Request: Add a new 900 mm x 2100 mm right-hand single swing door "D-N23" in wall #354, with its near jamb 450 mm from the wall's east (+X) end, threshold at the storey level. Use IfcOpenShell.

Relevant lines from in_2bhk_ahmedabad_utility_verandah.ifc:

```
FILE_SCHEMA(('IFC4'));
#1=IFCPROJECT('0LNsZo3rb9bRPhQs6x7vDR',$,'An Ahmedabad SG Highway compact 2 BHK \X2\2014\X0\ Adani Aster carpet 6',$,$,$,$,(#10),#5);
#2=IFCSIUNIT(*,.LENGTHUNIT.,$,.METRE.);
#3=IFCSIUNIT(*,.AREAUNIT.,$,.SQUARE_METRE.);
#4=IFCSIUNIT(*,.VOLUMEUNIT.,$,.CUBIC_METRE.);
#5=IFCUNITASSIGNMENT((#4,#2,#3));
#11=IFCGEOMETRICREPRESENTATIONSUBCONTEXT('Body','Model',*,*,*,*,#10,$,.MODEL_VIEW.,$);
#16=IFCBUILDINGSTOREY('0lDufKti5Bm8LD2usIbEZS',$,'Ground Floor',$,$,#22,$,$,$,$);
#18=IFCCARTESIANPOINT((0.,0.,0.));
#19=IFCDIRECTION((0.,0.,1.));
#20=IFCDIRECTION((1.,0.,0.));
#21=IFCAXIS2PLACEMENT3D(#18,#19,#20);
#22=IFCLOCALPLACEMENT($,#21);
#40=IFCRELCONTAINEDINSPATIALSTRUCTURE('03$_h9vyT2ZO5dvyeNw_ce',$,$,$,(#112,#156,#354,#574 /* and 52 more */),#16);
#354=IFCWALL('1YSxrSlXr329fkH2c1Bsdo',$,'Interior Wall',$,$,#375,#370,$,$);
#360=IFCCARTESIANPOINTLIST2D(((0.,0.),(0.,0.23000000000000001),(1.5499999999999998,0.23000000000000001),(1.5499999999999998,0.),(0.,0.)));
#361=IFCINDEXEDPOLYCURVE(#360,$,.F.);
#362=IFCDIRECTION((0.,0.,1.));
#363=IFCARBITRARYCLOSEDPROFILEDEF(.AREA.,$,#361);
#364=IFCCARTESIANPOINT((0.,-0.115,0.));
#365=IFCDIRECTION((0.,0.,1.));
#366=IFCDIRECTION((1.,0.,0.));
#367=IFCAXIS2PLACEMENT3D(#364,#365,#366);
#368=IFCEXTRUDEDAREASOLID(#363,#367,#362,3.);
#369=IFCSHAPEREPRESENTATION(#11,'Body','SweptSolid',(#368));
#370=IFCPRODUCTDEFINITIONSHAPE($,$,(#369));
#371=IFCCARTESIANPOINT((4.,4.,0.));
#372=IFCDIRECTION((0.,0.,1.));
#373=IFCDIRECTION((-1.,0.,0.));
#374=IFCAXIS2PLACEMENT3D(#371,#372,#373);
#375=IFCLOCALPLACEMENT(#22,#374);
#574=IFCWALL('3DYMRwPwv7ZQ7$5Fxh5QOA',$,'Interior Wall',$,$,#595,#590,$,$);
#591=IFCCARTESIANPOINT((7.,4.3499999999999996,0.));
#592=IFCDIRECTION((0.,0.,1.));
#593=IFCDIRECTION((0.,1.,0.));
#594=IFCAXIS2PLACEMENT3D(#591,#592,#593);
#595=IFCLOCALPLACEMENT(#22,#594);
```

```python
import numpy as np
import ifcopenshell
import ifcopenshell.api.feature
import ifcopenshell.api.geometry
import ifcopenshell.api.root
import ifcopenshell.api.spatial
import ifcopenshell.geom
import ifcopenshell.util.element
import ifcopenshell.util.placement
import ifcopenshell.util.representation
import ifcopenshell.util.shape
import ifcopenshell.util.unit

model = ifcopenshell.open("in_2bhk_ahmedabad_utility_verandah.ifc")
unit_scale = ifcopenshell.util.unit.calculate_unit_scale(model)
settings = ifcopenshell.geom.settings()


def volume(element):
    """Net volume in cubic metres, openings subtracted."""
    shape = ifcopenshell.geom.create_shape(settings, element)
    return ifcopenshell.util.shape.get_volume(shape.geometry)


wall = model.by_id(354)
storey = ifcopenshell.util.element.get_container(wall, ifc_class="IfcBuildingStorey")
context = ifcopenshell.util.representation.get_context(model, "Model", "Body", "MODEL_VIEW")
before = volume(wall)

width, height, from_end, sill = 0.9, 2.1, 0.45, 0.0  # metres

# The wall runs along its own X axis, and the end named is its -X end.
wall_shape = ifcopenshell.geom.create_shape(settings, wall)
x, y, z = ifcopenshell.util.shape.get_vertices(wall_shape.geometry).T
start = x.min() + from_end
face, thickness = float(y.min()), float(y.max() - y.min())
wall_matrix = ifcopenshell.util.placement.get_local_placement(wall.ObjectPlacement)
level = ifcopenshell.util.placement.get_local_placement(storey.ObjectPlacement)[2, 3]


def in_wall(x, y):
    """Placement at x, y metres in the wall's axes, at sill height."""
    matrix = wall_matrix.copy()
    matrix[:, 3] = wall_matrix @ np.array([x / unit_scale, y / unit_scale, 0.0, 1.0])
    matrix[2, 3] = level + sill / unit_scale
    return matrix


# Opening: a box that overshoots both wall faces by 50 mm.
opening = ifcopenshell.api.root.create_entity(model, ifc_class="IfcOpeningElement", predefined_type="OPENING")
box = ifcopenshell.api.geometry.add_wall_representation(
    model, context=context, length=width, height=height, thickness=thickness + 0.1
)
ifcopenshell.api.geometry.assign_representation(model, product=opening, representation=box)
ifcopenshell.api.geometry.edit_object_placement(model, product=opening, matrix=in_wall(start, face - 0.05), is_si=False)
ifcopenshell.api.feature.add_feature(model, feature=opening, element=wall)

door = ifcopenshell.api.root.create_entity(model, ifc_class="IfcDoor", name="D-N23", predefined_type="DOOR")
door.OverallWidth, door.OverallHeight = width / unit_scale, height / unit_scale
door.OperationType = "SINGLE_SWING_RIGHT"
body = ifcopenshell.api.geometry.add_door_representation(
    model,
    context=context,
    overall_width=door.OverallWidth,
    overall_height=door.OverallHeight,
    operation_type="SINGLE_SWING_RIGHT",
    lining_properties={"LiningDepth": thickness / unit_scale, "ThresholdDepth": thickness / unit_scale},
)
ifcopenshell.api.geometry.assign_representation(model, product=door, representation=body)
ifcopenshell.api.spatial.assign_container(model, products=[door], relating_structure=storey)
ifcopenshell.api.feature.add_filling(model, opening=opening, element=door)

# The lining spans the wall, so the door starts at the wall face.
ifcopenshell.api.geometry.edit_object_placement(model, product=door, matrix=in_wall(start, face), is_si=False)

after = volume(wall)

print(f"wall volume {before:.3f} -> {after:.3f} m3")

model.write("in_2bhk_ahmedabad_utility_verandah-out.ifc")
```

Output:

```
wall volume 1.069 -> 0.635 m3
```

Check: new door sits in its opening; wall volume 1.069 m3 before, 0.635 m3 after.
